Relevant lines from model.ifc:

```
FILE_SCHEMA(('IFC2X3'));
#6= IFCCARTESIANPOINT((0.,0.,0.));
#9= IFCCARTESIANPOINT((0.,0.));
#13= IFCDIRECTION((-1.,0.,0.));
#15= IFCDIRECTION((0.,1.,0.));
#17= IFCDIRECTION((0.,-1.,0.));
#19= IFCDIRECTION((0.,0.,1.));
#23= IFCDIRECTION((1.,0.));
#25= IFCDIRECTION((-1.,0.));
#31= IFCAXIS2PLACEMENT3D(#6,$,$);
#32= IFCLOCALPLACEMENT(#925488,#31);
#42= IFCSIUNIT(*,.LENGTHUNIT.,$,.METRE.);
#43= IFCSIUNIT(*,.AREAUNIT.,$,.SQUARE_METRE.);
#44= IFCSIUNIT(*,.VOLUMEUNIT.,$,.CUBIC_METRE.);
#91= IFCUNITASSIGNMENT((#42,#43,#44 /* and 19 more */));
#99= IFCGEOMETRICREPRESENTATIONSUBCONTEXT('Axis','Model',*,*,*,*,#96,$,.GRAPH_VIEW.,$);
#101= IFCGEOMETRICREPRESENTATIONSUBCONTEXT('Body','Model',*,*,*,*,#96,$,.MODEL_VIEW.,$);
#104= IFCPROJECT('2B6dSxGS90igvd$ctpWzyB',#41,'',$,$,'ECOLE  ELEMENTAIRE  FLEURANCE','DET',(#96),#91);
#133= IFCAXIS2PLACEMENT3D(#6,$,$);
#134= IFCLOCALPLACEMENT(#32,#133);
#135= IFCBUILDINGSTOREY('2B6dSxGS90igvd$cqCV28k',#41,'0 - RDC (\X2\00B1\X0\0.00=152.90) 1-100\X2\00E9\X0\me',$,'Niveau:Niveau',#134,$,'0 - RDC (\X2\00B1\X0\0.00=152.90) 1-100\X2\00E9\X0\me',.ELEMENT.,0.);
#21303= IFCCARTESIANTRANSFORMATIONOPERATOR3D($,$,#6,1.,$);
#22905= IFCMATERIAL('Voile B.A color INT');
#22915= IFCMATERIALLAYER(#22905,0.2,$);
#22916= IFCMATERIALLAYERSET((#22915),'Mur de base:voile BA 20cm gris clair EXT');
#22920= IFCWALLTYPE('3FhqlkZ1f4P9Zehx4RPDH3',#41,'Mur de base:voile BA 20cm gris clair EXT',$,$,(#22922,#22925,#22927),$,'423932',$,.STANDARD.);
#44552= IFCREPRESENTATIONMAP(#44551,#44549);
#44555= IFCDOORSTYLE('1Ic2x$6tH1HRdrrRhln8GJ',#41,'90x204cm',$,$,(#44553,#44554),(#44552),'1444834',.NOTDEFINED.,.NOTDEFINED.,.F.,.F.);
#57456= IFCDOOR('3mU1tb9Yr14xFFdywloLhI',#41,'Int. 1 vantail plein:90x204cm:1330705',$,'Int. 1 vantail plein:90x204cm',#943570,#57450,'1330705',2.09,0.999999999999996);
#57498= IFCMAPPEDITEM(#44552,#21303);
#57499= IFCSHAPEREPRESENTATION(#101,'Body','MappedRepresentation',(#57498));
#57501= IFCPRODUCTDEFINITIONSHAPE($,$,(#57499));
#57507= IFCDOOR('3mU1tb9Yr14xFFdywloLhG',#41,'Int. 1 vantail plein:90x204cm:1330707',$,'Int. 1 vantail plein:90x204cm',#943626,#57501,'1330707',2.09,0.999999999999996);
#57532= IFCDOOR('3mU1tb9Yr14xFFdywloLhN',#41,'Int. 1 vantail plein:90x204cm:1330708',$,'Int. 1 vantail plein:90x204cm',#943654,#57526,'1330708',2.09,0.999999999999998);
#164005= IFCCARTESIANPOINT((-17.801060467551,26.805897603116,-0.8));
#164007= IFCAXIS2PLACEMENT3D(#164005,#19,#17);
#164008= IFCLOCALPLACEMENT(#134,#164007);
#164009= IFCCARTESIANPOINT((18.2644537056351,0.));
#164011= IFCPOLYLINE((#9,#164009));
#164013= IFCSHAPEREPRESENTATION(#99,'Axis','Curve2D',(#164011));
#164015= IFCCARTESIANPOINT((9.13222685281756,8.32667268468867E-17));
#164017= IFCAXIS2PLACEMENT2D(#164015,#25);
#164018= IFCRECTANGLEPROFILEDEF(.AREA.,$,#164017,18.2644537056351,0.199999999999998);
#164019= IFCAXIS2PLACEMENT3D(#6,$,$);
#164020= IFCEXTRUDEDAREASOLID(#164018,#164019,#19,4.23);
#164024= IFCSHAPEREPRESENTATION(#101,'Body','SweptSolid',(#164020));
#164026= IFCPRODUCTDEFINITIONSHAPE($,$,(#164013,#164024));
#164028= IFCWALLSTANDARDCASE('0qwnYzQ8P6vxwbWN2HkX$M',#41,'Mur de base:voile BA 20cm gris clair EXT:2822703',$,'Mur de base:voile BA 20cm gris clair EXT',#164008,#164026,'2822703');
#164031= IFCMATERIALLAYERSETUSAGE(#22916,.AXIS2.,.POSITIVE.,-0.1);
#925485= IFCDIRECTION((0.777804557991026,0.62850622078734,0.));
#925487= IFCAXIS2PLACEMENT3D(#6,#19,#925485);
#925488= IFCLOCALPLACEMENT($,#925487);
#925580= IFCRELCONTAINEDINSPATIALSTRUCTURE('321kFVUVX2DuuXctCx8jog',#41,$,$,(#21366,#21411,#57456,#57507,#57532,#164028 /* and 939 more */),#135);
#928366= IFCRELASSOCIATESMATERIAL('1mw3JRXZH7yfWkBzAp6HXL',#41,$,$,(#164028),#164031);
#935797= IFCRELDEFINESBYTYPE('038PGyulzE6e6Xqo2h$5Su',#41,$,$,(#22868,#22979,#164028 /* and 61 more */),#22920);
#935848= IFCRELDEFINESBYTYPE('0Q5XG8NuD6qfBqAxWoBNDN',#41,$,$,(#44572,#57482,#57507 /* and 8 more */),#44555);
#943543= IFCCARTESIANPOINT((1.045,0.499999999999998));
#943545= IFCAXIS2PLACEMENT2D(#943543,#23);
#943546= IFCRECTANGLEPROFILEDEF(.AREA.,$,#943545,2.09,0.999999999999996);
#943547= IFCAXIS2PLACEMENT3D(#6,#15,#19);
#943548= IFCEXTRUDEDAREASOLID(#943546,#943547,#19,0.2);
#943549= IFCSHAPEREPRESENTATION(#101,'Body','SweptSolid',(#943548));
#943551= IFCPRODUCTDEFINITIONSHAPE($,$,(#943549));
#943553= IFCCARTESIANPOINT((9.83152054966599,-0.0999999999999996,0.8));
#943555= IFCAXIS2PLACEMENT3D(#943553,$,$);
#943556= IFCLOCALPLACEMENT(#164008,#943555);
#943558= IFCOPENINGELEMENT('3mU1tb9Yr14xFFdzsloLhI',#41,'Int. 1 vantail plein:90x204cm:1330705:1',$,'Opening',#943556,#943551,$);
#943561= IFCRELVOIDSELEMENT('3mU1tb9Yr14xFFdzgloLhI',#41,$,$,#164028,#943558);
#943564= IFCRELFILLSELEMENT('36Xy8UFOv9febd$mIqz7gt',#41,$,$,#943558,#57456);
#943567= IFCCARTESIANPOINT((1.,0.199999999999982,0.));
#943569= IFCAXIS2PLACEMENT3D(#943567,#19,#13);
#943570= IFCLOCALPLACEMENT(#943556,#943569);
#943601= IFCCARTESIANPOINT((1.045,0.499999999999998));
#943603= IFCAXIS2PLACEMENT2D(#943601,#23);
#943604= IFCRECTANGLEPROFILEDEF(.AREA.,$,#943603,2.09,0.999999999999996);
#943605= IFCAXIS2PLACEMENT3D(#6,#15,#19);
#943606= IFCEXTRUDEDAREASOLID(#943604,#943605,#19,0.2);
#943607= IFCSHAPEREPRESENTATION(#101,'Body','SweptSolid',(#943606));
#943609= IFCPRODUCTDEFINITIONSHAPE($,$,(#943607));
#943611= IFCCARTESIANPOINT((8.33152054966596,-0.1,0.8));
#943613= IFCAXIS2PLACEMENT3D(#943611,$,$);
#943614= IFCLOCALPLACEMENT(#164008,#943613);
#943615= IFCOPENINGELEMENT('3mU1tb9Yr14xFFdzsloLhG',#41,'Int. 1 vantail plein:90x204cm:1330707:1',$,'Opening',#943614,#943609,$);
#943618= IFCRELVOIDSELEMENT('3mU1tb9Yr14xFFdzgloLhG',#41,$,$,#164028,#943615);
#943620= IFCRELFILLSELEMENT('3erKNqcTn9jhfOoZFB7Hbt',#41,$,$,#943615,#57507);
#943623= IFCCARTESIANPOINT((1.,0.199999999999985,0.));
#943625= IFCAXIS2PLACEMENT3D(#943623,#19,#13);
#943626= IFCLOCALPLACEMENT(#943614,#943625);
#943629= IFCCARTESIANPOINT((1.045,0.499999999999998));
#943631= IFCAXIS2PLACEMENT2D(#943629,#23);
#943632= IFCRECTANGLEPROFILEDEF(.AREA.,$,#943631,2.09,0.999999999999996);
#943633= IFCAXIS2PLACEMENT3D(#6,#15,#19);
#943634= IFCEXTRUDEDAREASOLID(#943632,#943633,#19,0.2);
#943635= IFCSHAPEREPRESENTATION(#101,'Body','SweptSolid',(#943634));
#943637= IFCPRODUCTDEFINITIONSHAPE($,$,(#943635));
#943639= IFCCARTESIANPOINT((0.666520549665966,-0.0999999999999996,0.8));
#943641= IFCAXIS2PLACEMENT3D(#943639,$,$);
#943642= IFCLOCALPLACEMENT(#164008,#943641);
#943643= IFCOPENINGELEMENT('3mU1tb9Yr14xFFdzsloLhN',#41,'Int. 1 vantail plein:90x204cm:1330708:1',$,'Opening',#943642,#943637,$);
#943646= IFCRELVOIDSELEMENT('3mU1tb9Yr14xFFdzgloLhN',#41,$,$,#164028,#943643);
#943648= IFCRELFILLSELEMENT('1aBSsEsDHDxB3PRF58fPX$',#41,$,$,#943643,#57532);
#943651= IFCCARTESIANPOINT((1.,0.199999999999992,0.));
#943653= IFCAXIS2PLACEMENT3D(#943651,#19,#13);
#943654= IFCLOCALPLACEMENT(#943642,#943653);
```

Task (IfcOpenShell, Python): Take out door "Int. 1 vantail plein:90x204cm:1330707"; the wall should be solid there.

```python
import ifcopenshell
import ifcopenshell.api.feature
import ifcopenshell.api.root
import ifcopenshell.geom
import ifcopenshell.util.shape

model = ifcopenshell.open("model.ifc")
settings = ifcopenshell.geom.settings()


def volume(element):
    """Net volume in cubic metres, openings subtracted."""
    shape = ifcopenshell.geom.create_shape(settings, element)
    return ifcopenshell.util.shape.get_volume(shape.geometry)


door = model.by_id(57507)
opening = door.FillsVoids[0].RelatingOpeningElement
wall = opening.VoidsElements[0].RelatingBuildingElement
before = volume(wall)

ifcopenshell.api.root.remove_product(model, product=door)
ifcopenshell.api.feature.remove_feature(model, feature=opening)

after = volume(wall)

print(f"wall volume {before:.3f} -> {after:.3f} m3")

model.write("model_rev.ifc")
```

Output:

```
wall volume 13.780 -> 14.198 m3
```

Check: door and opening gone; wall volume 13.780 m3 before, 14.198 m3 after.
